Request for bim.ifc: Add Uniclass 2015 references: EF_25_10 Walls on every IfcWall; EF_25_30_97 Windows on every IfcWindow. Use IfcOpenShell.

First a look at what the model holds.

```python
import ifcopenshell

model = ifcopenshell.open("bim.ifc")
print(model.schema)
print("classifications:", [c.Name for c in model.by_type("IfcClassification")])
for ifc_class in ("IfcDoor", "IfcRoof", "IfcStair", "IfcWall", "IfcWindow"):
    print(ifc_class, len(model.by_type(ifc_class)))
```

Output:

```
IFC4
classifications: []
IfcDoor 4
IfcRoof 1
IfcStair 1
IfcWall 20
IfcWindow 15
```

```python
import ifcopenshell
import ifcopenshell.api.classification

model = ifcopenshell.open("bim.ifc")

system = ifcopenshell.api.classification.add_classification(model, classification="Uniclass 2015")

codes = {
    "IfcWall": ("EF_25_10", "Walls"),
    "IfcWindow": ("EF_25_30_97", "Windows"),
}
for ifc_class, (code, name) in codes.items():
    products = model.by_type(ifc_class)
    ifcopenshell.api.classification.add_reference(
        model, products=products, classification=system, identification=code, name=name
    )
    print(code, len(products))

model.write("bim_updated.ifc")
```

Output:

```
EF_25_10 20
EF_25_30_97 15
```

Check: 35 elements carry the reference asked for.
